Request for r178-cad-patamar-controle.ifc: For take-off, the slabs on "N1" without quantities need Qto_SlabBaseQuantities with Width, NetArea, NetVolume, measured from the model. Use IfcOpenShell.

First a look at what the model holds.

```python
import ifcopenshell
import ifcopenshell.util.element
import ifcopenshell.util.unit

model = ifcopenshell.open("r178-cad-patamar-controle.ifc")
print(model.schema)
for unit_type in ("LENGTHUNIT", "AREAUNIT", "VOLUMEUNIT"):
    print(unit_type, ifcopenshell.util.unit.calculate_unit_scale(model, unit_type))
storey = next(s for s in model.by_type("IfcBuildingStorey") if s.Name == "N1")
slabs = [e for e in ifcopenshell.util.element.get_decomposition(storey) if e.is_a("IfcSlab")]
for e in sorted(slabs, key=lambda e: e.id()):
    print(e.id(), e.is_a(), e.Name, list(ifcopenshell.util.element.get_psets(e, qtos_only=True)), sep=" | ")
```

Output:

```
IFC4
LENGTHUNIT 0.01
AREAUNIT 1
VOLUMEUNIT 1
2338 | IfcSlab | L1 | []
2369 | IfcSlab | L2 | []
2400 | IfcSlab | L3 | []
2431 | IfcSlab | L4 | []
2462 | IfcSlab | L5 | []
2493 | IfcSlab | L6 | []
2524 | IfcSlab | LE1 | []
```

```python
import ifcopenshell
import ifcopenshell.api.pset
import ifcopenshell.geom
import ifcopenshell.util.element
import ifcopenshell.util.shape
import ifcopenshell.util.unit

model = ifcopenshell.open("r178-cad-patamar-controle.ifc")
unit_scale = ifcopenshell.util.unit.calculate_unit_scale(model)
area_scale = ifcopenshell.util.unit.calculate_unit_scale(model, "AREAUNIT")
volume_scale = ifcopenshell.util.unit.calculate_unit_scale(model, "VOLUMEUNIT")
settings = ifcopenshell.geom.settings()

storey = next(s for s in model.by_type("IfcBuildingStorey") if s.Name == "N1")
slabs = [e for e in ifcopenshell.util.element.get_decomposition(storey) if e.is_a("IfcSlab")]

for e in sorted(slabs, key=lambda e: e.id()):
    if ifcopenshell.util.element.get_psets(e, qtos_only=True, should_inherit=False):
        continue
    # Geometry comes back in metres, in the element's own axes.
    shape = ifcopenshell.geom.create_shape(settings, e)
    values = {
        "Width": ifcopenshell.util.shape.get_z(shape.geometry) / unit_scale,
        "NetArea": ifcopenshell.util.shape.get_footprint_area(shape.geometry) / area_scale,
        "NetVolume": ifcopenshell.util.shape.get_volume(shape.geometry) / volume_scale,
    }
    qto = ifcopenshell.api.pset.add_qto(model, product=e, name="Qto_SlabBaseQuantities")
    ifcopenshell.api.pset.edit_qto(model, qto=qto, properties=values)
    print(e.id(), {k: round(v, 3) for k, v in values.items()})

model.write("r178-cad-patamar-controle_rev.ifc")
```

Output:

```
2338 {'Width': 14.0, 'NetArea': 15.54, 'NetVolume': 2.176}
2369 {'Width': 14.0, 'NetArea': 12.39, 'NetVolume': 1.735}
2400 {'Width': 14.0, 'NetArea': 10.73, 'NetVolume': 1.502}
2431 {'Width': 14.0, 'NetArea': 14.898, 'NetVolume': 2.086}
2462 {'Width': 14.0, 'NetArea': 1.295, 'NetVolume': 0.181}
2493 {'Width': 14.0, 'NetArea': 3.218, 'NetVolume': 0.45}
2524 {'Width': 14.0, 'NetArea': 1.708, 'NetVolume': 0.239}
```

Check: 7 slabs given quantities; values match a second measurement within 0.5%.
